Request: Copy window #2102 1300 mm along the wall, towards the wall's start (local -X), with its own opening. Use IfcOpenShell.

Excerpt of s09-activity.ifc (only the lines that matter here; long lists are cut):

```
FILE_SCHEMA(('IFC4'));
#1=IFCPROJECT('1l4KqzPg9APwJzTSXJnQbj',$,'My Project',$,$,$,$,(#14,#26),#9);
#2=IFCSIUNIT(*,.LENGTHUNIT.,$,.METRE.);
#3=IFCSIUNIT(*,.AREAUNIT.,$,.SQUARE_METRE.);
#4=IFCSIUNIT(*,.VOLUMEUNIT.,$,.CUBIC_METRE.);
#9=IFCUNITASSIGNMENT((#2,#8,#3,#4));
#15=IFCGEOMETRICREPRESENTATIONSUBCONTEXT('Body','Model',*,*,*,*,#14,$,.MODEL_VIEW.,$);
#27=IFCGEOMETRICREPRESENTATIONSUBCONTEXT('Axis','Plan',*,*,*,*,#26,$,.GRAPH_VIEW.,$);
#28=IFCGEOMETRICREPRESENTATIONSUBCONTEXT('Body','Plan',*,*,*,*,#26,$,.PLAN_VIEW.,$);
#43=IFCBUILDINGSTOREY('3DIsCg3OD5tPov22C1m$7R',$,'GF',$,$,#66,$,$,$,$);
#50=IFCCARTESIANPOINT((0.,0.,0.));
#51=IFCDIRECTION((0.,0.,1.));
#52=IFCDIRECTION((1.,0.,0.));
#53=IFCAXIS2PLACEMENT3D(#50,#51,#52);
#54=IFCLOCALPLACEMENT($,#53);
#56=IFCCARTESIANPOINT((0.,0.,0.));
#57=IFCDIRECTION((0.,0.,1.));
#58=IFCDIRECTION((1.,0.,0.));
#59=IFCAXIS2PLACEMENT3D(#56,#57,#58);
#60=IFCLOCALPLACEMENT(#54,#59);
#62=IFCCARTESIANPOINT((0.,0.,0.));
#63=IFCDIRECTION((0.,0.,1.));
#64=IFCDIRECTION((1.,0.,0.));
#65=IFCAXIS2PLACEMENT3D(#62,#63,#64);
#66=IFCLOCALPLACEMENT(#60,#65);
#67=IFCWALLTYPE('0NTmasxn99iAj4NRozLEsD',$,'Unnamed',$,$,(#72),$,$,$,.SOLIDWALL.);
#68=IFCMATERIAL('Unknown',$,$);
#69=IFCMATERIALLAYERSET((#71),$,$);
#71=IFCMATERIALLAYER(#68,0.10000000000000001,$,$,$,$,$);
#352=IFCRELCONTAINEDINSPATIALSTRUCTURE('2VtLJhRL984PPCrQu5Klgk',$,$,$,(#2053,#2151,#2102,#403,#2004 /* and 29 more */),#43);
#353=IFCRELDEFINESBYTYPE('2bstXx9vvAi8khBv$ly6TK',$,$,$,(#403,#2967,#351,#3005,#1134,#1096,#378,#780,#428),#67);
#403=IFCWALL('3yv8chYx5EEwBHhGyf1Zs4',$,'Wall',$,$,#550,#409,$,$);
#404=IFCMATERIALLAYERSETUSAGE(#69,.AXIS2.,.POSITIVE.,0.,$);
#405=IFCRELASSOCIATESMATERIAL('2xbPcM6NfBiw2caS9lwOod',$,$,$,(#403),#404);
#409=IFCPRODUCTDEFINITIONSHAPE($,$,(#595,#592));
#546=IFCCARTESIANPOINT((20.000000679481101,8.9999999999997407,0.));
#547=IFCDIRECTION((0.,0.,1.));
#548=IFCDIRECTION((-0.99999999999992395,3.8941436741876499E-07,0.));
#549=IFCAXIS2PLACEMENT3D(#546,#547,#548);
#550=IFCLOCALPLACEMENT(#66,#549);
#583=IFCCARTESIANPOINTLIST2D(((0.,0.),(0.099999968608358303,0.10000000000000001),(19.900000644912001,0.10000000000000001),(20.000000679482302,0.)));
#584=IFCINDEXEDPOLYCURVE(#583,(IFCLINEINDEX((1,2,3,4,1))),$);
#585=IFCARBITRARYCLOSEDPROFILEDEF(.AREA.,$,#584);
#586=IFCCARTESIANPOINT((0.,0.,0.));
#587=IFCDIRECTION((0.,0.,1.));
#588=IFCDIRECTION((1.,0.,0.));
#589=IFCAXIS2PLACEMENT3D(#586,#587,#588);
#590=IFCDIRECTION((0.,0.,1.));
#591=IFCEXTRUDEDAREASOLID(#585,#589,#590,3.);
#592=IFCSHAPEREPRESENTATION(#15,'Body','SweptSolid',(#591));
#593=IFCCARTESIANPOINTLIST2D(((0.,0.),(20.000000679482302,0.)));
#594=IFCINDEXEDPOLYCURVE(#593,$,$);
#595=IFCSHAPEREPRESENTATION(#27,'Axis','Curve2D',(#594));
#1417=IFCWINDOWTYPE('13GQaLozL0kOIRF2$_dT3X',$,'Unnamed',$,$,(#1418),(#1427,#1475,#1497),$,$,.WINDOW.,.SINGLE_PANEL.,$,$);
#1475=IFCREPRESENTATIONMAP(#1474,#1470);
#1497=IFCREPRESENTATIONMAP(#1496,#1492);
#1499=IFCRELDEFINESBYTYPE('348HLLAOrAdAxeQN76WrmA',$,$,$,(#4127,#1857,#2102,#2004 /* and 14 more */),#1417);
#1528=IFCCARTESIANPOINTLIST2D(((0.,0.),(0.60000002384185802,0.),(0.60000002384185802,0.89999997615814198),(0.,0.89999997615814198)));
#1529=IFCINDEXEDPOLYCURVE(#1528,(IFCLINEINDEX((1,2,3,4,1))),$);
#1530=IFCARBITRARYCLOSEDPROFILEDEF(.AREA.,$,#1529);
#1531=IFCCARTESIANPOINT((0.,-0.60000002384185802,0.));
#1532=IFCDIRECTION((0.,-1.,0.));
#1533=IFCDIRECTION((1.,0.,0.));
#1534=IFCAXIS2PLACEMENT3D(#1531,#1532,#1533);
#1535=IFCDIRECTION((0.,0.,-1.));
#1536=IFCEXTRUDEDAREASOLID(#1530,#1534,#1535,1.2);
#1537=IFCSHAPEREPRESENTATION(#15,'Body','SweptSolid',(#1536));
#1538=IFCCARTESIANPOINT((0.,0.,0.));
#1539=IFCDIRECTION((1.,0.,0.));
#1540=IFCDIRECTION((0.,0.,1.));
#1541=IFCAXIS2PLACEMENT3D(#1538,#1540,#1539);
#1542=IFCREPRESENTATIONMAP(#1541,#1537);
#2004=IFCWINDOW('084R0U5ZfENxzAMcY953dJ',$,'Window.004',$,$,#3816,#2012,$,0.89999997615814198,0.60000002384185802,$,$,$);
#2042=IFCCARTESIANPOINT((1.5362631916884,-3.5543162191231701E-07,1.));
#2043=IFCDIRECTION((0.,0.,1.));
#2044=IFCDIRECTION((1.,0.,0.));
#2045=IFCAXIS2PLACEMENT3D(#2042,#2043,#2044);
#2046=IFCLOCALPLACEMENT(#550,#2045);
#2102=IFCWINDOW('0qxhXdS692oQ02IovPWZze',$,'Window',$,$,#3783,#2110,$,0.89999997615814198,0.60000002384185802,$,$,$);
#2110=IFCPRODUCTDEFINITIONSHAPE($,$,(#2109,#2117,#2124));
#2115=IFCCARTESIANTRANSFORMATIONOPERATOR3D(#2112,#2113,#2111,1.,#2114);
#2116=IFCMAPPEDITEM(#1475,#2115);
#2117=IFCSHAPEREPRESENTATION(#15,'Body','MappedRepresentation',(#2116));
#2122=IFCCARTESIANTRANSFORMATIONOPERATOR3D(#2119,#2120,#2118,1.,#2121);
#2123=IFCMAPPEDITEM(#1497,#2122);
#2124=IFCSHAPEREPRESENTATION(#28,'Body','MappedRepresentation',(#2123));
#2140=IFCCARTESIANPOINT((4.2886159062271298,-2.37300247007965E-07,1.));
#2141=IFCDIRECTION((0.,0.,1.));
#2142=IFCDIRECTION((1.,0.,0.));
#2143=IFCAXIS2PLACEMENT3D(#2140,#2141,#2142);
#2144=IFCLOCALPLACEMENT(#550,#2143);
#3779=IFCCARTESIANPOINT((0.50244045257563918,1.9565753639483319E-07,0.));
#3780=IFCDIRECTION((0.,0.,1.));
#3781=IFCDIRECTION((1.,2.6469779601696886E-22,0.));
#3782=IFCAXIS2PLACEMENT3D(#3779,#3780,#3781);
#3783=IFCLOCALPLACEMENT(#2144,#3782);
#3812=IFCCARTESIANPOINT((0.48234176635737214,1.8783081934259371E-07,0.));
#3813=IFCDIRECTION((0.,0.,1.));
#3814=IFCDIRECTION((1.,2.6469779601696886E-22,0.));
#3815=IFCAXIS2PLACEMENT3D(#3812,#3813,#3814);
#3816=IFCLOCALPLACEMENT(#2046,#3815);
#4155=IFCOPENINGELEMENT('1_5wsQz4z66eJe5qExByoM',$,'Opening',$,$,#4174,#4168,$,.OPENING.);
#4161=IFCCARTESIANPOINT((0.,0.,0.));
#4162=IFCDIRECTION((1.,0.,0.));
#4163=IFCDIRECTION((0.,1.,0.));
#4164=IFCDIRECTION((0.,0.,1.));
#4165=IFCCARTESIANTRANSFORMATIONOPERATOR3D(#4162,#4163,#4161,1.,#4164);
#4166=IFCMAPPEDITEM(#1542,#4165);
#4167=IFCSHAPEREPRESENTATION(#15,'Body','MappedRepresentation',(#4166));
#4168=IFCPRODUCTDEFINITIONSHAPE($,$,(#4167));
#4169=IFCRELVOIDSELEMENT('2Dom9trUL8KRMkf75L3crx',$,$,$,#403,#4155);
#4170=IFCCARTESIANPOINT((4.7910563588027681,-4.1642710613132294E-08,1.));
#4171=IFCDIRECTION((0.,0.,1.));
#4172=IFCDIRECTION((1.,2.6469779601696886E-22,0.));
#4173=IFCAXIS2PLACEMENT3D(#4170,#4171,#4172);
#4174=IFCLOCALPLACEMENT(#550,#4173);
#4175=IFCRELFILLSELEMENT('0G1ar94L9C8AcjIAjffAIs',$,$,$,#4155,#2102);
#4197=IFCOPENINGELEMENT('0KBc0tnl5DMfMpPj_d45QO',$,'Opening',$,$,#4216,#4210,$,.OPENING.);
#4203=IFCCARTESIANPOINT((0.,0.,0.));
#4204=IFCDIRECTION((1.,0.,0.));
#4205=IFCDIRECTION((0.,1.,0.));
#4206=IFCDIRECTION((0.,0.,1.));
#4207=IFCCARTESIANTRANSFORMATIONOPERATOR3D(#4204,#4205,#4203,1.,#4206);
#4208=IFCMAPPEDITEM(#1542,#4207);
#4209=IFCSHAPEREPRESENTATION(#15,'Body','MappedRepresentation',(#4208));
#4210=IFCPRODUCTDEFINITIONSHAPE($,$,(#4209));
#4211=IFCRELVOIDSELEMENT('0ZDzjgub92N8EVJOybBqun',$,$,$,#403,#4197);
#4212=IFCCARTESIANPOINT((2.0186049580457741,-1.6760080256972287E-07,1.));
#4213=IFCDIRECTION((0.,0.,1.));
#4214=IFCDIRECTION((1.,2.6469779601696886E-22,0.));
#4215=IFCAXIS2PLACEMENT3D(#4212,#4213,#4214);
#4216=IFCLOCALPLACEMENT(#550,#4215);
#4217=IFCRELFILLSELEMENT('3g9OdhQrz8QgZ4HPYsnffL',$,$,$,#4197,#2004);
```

```python
import ifcopenshell
import ifcopenshell.api.feature
import ifcopenshell.api.geometry
import ifcopenshell.api.root
import ifcopenshell.geom
import ifcopenshell.util.element
import ifcopenshell.util.placement
import ifcopenshell.util.shape
import ifcopenshell.util.unit

model = ifcopenshell.open("s09-activity.ifc")
unit_scale = ifcopenshell.util.unit.calculate_unit_scale(model)
settings = ifcopenshell.geom.settings()


def volume(element):
    """Net volume in cubic metres, openings subtracted."""
    shape = ifcopenshell.geom.create_shape(settings, element)
    return ifcopenshell.util.shape.get_volume(shape.geometry)


window = model.by_guid("0qxhXdS692oQ02IovPWZze")
opening = window.FillsVoids[0].RelatingOpeningElement
wall = opening.VoidsElements[0].RelatingBuildingElement
before = volume(wall)
shift = ifcopenshell.util.placement.get_local_placement(wall.ObjectPlacement)[:3, 0] * -1.3 / unit_scale

# copy_class copies the void relationship, type, container and properties, but no geometry.
new_opening = ifcopenshell.api.root.copy_class(model, product=opening)
new_opening.Representation = ifcopenshell.util.element.copy_deep(
    model, opening.Representation, exclude=["IfcGeometricRepresentationContext", "IfcRepresentationMap"]
)
new_window = ifcopenshell.api.root.copy_class(model, product=window)
new_window.Representation = ifcopenshell.util.element.copy_deep(
    model, window.Representation, exclude=["IfcGeometricRepresentationContext", "IfcRepresentationMap"]
)
ifcopenshell.api.feature.add_filling(model, opening=new_opening, element=new_window)

for old, new in ((opening, new_opening), (window, new_window)):
    matrix = ifcopenshell.util.placement.get_local_placement(old.ObjectPlacement)
    matrix[:3, 3] += shift
    ifcopenshell.api.geometry.edit_object_placement(model, product=new, matrix=matrix, is_si=False)

after = volume(wall)

print(f"wall volume {before:.3f} -> {after:.3f} m3")

model.write("s09-activity_updated.ifc")
```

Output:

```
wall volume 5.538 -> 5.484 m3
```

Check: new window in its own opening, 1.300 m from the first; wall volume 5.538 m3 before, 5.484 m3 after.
